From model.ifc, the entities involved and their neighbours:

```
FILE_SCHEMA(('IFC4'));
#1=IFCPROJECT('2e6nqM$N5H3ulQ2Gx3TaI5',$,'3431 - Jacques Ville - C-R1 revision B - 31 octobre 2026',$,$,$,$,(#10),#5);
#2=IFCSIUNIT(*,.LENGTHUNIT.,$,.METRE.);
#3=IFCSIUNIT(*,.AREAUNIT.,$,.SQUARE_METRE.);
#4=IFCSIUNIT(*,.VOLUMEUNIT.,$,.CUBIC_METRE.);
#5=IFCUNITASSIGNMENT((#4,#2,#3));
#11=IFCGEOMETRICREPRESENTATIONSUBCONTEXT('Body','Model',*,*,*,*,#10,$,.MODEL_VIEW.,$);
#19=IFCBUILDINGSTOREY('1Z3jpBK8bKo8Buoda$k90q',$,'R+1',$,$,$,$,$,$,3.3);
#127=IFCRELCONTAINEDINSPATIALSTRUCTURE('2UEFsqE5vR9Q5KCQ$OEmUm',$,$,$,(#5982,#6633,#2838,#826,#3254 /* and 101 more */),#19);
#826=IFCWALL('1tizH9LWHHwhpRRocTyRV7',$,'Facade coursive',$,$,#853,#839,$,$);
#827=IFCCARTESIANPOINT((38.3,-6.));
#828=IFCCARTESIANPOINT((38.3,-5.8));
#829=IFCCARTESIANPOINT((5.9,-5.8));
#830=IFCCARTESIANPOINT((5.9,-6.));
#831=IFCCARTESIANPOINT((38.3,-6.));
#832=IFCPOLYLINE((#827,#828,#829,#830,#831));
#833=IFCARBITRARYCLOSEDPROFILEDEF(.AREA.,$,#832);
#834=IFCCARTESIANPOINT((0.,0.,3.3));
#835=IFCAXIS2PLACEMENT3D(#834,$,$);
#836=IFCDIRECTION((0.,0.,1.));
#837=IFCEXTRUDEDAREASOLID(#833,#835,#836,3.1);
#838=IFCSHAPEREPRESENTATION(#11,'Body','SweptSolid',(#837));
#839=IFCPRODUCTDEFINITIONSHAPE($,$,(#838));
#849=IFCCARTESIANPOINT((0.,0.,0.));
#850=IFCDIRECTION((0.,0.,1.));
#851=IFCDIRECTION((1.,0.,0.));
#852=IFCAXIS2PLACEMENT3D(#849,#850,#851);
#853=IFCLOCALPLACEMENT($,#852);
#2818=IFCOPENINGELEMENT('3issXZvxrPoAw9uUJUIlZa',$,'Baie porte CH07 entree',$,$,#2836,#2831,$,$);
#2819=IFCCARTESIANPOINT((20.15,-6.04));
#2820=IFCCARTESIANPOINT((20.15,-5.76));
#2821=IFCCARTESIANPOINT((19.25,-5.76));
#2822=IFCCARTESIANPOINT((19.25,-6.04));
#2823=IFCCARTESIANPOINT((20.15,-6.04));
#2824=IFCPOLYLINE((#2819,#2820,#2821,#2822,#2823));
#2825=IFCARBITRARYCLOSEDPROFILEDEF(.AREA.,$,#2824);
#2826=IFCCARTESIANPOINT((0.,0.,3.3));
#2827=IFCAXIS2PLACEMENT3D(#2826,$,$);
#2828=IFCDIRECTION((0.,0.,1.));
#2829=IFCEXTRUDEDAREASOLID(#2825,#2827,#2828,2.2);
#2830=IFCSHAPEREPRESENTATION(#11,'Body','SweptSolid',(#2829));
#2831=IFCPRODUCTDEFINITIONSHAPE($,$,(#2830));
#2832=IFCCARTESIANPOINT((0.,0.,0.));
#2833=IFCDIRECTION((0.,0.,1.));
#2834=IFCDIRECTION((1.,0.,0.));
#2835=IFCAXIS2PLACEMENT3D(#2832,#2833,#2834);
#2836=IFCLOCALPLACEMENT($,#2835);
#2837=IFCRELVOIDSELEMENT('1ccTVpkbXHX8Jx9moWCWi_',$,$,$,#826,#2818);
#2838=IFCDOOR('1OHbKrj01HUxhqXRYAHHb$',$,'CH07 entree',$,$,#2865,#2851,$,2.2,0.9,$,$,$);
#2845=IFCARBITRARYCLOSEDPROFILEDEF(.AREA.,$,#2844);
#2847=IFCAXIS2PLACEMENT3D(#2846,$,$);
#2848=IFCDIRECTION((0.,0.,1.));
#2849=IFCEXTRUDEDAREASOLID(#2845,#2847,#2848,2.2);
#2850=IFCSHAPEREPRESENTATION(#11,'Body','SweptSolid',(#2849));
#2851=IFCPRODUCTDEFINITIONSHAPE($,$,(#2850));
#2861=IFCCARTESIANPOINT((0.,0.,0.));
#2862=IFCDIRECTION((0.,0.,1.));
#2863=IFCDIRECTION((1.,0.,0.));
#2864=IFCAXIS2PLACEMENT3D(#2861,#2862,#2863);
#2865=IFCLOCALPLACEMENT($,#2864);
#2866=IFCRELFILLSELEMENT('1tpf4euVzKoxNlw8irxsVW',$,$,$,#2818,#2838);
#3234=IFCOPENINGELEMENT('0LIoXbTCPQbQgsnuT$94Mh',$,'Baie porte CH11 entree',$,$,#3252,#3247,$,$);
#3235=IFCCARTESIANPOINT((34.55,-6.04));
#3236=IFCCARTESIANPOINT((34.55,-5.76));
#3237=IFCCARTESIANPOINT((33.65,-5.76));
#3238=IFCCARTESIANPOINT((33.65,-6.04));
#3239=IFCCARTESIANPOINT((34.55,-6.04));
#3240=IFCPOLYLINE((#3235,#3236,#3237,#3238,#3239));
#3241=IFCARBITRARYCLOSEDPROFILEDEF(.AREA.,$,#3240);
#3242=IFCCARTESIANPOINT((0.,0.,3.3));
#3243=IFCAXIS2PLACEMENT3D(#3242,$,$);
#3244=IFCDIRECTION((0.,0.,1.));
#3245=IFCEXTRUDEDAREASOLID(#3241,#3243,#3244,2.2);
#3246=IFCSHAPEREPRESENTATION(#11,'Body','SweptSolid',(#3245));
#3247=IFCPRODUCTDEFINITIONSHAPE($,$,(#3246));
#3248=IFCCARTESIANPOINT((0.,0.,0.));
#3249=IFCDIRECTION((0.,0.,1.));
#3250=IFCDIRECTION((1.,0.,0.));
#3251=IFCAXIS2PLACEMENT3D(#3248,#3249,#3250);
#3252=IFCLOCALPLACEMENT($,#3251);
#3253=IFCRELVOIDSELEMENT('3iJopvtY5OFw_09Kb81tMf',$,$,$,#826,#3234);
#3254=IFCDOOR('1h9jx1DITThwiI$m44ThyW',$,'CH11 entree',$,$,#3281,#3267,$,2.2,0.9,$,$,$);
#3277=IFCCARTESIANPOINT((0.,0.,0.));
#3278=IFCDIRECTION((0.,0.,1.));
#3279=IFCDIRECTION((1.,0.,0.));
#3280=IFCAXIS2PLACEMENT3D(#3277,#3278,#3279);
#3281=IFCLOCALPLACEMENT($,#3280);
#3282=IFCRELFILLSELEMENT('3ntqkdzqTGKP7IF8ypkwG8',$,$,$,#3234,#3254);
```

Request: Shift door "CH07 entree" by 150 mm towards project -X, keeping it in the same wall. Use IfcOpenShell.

```python
import ifcopenshell
import ifcopenshell.api.geometry
import ifcopenshell.util.placement

model = ifcopenshell.open("model.ifc")

door = model.by_guid("1OHbKrj01HUxhqXRYAHHb$")
opening = door.FillsVoids[0].RelatingOpeningElement
wall = opening.VoidsElements[0].RelatingBuildingElement

wall_matrix = ifcopenshell.util.placement.get_local_placement(wall.ObjectPlacement)
shift = wall_matrix[:3, 0] * -0.15
before = ifcopenshell.util.placement.get_local_placement(door.ObjectPlacement)[:3, 3].copy()

# The door is not placed relative to its opening, so move both.
for product in (opening, door):
    matrix = ifcopenshell.util.placement.get_local_placement(product.ObjectPlacement)
    matrix[:3, 3] += shift
    ifcopenshell.api.geometry.edit_object_placement(model, product=product, matrix=matrix, is_si=False)

after = ifcopenshell.util.placement.get_local_placement(door.ObjectPlacement)[:3, 3]
print("door moved by", (after - before).round(3) + 0.0)

model.write("model-out.ifc")
```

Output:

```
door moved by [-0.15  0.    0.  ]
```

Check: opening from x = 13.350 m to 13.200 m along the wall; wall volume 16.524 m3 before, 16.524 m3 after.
